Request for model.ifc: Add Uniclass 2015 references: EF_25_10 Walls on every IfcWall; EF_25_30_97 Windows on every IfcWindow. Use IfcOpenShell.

First a look at what the model holds.

```python
import ifcopenshell

model = ifcopenshell.open("model.ifc")
print(model.schema)
print("classifications:", [c.Name for c in model.by_type("IfcClassification")])
for ifc_class in ("IfcDoor", "IfcRoof", "IfcStair", "IfcWall", "IfcWindow"):
    print(ifc_class, len(model.by_type(ifc_class)))
```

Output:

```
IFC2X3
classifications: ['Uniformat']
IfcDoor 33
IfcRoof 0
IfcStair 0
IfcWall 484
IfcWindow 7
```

```python
import ifcopenshell
import ifcopenshell.api.classification

model = ifcopenshell.open("model.ifc")

# IFC2X3 requires Source and Edition and has no link from the project to the system.
system = model.create_entity("IfcClassification", Source="NBS", Edition="2015", Name="Uniclass 2015")

codes = {
    "IfcWall": ("EF_25_10", "Walls"),
    "IfcWindow": ("EF_25_30_97", "Windows"),
}
for ifc_class, (code, name) in codes.items():
    products = model.by_type(ifc_class)
    ifcopenshell.api.classification.add_reference(
        model, products=products, classification=system, identification=code, name=name
    )
    print(code, len(products))

model.write("model-out.ifc")
```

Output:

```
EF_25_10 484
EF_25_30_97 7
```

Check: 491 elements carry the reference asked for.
